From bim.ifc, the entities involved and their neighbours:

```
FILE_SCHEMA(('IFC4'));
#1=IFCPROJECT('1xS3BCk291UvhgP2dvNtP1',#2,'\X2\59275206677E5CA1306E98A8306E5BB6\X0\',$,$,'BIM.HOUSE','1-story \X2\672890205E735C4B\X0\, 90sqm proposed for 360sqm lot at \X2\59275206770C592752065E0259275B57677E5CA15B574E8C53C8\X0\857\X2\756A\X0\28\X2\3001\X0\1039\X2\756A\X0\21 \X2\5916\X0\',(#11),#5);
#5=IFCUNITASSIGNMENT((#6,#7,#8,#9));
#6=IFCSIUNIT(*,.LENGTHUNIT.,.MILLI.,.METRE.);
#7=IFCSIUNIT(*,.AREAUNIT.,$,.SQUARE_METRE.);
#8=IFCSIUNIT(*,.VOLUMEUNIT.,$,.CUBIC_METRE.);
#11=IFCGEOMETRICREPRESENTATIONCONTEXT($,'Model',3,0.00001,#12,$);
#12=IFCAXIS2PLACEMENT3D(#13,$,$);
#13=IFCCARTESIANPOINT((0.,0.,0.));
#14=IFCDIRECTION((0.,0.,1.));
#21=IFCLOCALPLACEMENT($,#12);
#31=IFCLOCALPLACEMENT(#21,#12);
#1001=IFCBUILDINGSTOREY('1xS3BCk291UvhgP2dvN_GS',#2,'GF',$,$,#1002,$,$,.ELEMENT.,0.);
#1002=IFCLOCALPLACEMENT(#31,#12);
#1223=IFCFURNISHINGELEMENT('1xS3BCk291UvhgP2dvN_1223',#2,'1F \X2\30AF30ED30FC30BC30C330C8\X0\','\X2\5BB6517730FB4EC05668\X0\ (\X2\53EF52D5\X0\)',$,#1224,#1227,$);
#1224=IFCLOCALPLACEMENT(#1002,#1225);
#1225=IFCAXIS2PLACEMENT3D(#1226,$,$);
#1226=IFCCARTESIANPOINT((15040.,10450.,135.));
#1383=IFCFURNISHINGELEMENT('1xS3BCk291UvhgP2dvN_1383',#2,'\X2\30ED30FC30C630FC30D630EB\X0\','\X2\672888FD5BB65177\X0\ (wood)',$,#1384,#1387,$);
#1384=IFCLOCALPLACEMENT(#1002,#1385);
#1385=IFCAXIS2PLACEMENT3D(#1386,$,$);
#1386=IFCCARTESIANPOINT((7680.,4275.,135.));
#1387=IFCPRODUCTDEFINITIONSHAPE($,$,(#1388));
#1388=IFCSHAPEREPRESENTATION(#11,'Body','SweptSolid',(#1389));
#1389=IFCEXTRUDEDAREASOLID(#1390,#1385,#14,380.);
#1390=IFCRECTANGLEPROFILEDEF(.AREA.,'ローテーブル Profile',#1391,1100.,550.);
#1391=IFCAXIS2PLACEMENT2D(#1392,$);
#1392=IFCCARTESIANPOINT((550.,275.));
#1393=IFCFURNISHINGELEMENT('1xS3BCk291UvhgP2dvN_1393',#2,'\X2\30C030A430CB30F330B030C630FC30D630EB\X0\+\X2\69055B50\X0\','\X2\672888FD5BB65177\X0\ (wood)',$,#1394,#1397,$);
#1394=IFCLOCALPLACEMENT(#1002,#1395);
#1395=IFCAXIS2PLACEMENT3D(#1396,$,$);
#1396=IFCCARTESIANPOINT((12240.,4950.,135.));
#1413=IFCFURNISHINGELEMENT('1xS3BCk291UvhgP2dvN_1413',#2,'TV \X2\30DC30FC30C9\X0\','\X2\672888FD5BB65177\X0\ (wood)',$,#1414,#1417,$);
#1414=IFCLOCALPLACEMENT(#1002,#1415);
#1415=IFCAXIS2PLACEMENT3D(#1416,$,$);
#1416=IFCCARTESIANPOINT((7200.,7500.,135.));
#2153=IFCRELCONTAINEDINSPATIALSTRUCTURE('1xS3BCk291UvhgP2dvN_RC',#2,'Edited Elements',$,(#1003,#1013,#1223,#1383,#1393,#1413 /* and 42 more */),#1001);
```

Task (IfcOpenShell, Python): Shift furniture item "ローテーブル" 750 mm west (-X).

```python
import ifcopenshell
import ifcopenshell.api.geometry
import ifcopenshell.util.placement
import ifcopenshell.util.unit

model = ifcopenshell.open("bim.ifc")
unit_scale = ifcopenshell.util.unit.calculate_unit_scale(model)

item = model.by_guid("1xS3BCk291UvhgP2dvN_1383")
matrix = ifcopenshell.util.placement.get_local_placement(item.ObjectPlacement)
matrix[0, 3] -= 0.75 / unit_scale
ifcopenshell.api.geometry.edit_object_placement(model, product=item, matrix=matrix, is_si=False)

print(ifcopenshell.util.placement.get_local_placement(item.ObjectPlacement).round(3) + 0.0)

model.write("bim_updated.ifc")
```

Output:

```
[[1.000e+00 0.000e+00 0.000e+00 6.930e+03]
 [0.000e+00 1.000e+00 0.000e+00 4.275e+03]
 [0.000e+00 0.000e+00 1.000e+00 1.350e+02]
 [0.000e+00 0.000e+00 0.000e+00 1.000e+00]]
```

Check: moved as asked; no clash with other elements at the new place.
